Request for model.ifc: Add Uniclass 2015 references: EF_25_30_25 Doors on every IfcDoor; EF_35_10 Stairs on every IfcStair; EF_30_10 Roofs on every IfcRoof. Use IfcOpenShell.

First a look at what the model holds.

```python
import ifcopenshell

model = ifcopenshell.open("model.ifc")
print(model.schema)
print("classifications:", [c.Name for c in model.by_type("IfcClassification")])
for ifc_class in ("IfcDoor", "IfcRoof", "IfcStair", "IfcWall", "IfcWindow"):
    print(ifc_class, len(model.by_type(ifc_class)))
```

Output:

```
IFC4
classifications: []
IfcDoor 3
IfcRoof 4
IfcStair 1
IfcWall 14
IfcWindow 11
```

```python
import ifcopenshell
import ifcopenshell.api.classification

model = ifcopenshell.open("model.ifc")

system = ifcopenshell.api.classification.add_classification(model, classification="Uniclass 2015")

codes = {
    "IfcDoor": ("EF_25_30_25", "Doors"),
    "IfcStair": ("EF_35_10", "Stairs"),
    "IfcRoof": ("EF_30_10", "Roofs"),
}
for ifc_class, (code, name) in codes.items():
    products = model.by_type(ifc_class)
    ifcopenshell.api.classification.add_reference(
        model, products=products, classification=system, identification=code, name=name
    )
    print(code, len(products))

model.write("model_edited.ifc")
```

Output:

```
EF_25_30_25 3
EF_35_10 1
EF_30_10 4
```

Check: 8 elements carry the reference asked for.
